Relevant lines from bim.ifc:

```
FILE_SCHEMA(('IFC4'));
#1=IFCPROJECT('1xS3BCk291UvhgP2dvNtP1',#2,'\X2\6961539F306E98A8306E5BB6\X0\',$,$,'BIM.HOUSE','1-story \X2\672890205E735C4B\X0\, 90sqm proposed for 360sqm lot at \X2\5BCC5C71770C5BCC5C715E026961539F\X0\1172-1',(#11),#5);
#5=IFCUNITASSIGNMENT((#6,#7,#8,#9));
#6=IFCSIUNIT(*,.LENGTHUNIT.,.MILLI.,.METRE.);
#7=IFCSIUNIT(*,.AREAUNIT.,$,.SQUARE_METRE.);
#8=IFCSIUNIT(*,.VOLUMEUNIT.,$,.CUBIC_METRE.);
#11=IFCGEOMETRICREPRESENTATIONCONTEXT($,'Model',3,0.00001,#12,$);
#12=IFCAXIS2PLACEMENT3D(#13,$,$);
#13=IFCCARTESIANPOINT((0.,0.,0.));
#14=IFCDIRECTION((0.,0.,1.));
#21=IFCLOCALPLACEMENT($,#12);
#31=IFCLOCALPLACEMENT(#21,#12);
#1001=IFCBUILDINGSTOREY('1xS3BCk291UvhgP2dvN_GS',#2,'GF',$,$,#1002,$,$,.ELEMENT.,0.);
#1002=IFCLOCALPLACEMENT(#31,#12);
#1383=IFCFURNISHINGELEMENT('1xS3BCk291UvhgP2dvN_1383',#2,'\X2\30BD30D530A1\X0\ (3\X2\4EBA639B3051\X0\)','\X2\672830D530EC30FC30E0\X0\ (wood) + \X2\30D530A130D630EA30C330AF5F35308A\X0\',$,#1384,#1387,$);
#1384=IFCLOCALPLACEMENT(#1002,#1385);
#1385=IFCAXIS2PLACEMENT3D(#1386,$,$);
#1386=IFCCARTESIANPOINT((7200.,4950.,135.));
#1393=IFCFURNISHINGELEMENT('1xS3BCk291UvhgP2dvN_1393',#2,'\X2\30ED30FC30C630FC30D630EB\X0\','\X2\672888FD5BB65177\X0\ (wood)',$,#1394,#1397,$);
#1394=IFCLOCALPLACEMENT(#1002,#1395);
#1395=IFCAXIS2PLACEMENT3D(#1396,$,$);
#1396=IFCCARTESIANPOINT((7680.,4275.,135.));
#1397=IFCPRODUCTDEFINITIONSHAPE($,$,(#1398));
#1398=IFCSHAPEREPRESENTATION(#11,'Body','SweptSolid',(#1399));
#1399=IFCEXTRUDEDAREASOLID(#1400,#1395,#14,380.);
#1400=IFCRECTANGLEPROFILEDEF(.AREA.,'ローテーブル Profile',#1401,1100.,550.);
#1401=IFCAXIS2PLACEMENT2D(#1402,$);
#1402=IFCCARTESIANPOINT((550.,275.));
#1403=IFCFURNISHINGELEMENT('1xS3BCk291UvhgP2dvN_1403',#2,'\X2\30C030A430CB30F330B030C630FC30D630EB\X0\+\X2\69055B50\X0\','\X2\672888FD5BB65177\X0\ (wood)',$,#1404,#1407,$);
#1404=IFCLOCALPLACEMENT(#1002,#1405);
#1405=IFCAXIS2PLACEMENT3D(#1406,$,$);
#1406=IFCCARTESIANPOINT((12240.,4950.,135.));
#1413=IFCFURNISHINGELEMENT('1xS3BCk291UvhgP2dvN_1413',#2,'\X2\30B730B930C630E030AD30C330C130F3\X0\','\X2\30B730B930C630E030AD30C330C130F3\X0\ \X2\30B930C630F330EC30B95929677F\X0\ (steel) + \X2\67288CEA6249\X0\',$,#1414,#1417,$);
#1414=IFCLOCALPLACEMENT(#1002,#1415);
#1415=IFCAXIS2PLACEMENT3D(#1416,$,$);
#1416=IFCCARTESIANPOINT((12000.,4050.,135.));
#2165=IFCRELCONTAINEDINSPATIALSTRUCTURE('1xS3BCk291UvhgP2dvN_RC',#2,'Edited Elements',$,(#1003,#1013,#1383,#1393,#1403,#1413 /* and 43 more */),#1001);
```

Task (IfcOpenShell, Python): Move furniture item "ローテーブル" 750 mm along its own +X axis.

```python
import ifcopenshell
import ifcopenshell.api.geometry
import ifcopenshell.util.placement
import ifcopenshell.util.unit

model = ifcopenshell.open("bim.ifc")
unit_scale = ifcopenshell.util.unit.calculate_unit_scale(model)

item = model.by_guid("1xS3BCk291UvhgP2dvN_1393")
matrix = ifcopenshell.util.placement.get_local_placement(item.ObjectPlacement)
matrix[:3, 3] += matrix[:3, 0] * 0.75 / unit_scale
ifcopenshell.api.geometry.edit_object_placement(model, product=item, matrix=matrix, is_si=False)

print(ifcopenshell.util.placement.get_local_placement(item.ObjectPlacement).round(3) + 0.0)

model.write("bim_updated.ifc")
```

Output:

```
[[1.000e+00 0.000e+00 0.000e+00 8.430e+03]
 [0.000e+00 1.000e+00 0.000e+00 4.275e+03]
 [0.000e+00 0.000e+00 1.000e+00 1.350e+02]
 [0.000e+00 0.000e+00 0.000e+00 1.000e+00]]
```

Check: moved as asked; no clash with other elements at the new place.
